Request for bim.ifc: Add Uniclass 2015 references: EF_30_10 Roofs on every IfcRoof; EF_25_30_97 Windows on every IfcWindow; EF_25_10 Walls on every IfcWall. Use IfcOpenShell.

First a look at what the model holds.

```python
import ifcopenshell

model = ifcopenshell.open("bim.ifc")
print(model.schema)
print("classifications:", [c.Name for c in model.by_type("IfcClassification")])
for ifc_class in ("IfcDoor", "IfcRoof", "IfcStair", "IfcWall", "IfcWindow"):
    print(ifc_class, len(model.by_type(ifc_class)))
```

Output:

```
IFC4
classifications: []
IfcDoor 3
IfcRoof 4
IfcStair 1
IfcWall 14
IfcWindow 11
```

```python
import ifcopenshell
import ifcopenshell.api.classification

model = ifcopenshell.open("bim.ifc")

system = ifcopenshell.api.classification.add_classification(model, classification="Uniclass 2015")

codes = {
    "IfcRoof": ("EF_30_10", "Roofs"),
    "IfcWindow": ("EF_25_30_97", "Windows"),
    "IfcWall": ("EF_25_10", "Walls"),
}
for ifc_class, (code, name) in codes.items():
    products = model.by_type(ifc_class)
    ifcopenshell.api.classification.add_reference(
        model, products=products, classification=system, identification=code, name=name
    )
    print(code, len(products))

model.write("bim_updated.ifc")
```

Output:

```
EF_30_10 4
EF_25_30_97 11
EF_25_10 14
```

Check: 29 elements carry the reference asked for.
